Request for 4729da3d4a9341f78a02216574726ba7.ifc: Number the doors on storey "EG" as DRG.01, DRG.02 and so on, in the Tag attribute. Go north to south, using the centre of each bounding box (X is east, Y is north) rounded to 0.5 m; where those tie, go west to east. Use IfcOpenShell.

First a look at what the model holds.

```python
import ifcopenshell
import ifcopenshell.util.element
import ifcopenshell.util.placement

model = ifcopenshell.open("4729da3d4a9341f78a02216574726ba7.ifc")
print(model.schema)
storey = next(s for s in model.by_type("IfcBuildingStorey") if s.Name == "EG")
doors = [e for e in ifcopenshell.util.element.get_decomposition(storey) if e.is_a("IfcDoor")]
for e in sorted(doors, key=lambda e: e.id()):
    origin = ifcopenshell.util.placement.get_local_placement(e.ObjectPlacement)[:3, 3]
    print(e.id(), e.Tag, e.Name, origin.round(2) + 0.0, sep=" | ")
```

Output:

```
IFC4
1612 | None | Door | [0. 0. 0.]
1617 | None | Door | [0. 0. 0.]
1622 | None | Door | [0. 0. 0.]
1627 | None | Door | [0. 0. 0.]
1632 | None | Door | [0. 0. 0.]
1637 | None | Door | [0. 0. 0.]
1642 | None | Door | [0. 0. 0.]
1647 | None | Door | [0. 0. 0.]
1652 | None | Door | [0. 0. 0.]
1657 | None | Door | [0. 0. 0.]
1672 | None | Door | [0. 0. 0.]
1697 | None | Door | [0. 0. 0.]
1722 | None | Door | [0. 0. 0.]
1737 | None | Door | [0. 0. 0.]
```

```python
import ifcopenshell
import ifcopenshell.geom
import ifcopenshell.util.element
import ifcopenshell.util.shape

model = ifcopenshell.open("4729da3d4a9341f78a02216574726ba7.ifc")
settings = ifcopenshell.geom.settings()
settings.set("use-world-coords", True)


def centre(element):
    shape = ifcopenshell.geom.create_shape(settings, element)
    return ifcopenshell.util.shape.get_bbox_centroid(shape.geometry)


storey = next(s for s in model.by_type("IfcBuildingStorey") if s.Name == "EG")
doors = [e for e in ifcopenshell.util.element.get_decomposition(storey) if e.is_a("IfcDoor")]

# Insertion points can sit at a corner or the storey origin, so sort by the geometry (in metres).
centres = {e: centre(e) for e in doors}
doors.sort(key=lambda e: (-round(centres[e][1] / 0.5), centres[e][0]))

for i, e in enumerate(doors, start=1):
    number = f"DRG.{i:02d}"
    e.Tag = number
    print(e.id(), number)

model.write("4729da3d4a9341f78a02216574726ba7_edited.ifc")
```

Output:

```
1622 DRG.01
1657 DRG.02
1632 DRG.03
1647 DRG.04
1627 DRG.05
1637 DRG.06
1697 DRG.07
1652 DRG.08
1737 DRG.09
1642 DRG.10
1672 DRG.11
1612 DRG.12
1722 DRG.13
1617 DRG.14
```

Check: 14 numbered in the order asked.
